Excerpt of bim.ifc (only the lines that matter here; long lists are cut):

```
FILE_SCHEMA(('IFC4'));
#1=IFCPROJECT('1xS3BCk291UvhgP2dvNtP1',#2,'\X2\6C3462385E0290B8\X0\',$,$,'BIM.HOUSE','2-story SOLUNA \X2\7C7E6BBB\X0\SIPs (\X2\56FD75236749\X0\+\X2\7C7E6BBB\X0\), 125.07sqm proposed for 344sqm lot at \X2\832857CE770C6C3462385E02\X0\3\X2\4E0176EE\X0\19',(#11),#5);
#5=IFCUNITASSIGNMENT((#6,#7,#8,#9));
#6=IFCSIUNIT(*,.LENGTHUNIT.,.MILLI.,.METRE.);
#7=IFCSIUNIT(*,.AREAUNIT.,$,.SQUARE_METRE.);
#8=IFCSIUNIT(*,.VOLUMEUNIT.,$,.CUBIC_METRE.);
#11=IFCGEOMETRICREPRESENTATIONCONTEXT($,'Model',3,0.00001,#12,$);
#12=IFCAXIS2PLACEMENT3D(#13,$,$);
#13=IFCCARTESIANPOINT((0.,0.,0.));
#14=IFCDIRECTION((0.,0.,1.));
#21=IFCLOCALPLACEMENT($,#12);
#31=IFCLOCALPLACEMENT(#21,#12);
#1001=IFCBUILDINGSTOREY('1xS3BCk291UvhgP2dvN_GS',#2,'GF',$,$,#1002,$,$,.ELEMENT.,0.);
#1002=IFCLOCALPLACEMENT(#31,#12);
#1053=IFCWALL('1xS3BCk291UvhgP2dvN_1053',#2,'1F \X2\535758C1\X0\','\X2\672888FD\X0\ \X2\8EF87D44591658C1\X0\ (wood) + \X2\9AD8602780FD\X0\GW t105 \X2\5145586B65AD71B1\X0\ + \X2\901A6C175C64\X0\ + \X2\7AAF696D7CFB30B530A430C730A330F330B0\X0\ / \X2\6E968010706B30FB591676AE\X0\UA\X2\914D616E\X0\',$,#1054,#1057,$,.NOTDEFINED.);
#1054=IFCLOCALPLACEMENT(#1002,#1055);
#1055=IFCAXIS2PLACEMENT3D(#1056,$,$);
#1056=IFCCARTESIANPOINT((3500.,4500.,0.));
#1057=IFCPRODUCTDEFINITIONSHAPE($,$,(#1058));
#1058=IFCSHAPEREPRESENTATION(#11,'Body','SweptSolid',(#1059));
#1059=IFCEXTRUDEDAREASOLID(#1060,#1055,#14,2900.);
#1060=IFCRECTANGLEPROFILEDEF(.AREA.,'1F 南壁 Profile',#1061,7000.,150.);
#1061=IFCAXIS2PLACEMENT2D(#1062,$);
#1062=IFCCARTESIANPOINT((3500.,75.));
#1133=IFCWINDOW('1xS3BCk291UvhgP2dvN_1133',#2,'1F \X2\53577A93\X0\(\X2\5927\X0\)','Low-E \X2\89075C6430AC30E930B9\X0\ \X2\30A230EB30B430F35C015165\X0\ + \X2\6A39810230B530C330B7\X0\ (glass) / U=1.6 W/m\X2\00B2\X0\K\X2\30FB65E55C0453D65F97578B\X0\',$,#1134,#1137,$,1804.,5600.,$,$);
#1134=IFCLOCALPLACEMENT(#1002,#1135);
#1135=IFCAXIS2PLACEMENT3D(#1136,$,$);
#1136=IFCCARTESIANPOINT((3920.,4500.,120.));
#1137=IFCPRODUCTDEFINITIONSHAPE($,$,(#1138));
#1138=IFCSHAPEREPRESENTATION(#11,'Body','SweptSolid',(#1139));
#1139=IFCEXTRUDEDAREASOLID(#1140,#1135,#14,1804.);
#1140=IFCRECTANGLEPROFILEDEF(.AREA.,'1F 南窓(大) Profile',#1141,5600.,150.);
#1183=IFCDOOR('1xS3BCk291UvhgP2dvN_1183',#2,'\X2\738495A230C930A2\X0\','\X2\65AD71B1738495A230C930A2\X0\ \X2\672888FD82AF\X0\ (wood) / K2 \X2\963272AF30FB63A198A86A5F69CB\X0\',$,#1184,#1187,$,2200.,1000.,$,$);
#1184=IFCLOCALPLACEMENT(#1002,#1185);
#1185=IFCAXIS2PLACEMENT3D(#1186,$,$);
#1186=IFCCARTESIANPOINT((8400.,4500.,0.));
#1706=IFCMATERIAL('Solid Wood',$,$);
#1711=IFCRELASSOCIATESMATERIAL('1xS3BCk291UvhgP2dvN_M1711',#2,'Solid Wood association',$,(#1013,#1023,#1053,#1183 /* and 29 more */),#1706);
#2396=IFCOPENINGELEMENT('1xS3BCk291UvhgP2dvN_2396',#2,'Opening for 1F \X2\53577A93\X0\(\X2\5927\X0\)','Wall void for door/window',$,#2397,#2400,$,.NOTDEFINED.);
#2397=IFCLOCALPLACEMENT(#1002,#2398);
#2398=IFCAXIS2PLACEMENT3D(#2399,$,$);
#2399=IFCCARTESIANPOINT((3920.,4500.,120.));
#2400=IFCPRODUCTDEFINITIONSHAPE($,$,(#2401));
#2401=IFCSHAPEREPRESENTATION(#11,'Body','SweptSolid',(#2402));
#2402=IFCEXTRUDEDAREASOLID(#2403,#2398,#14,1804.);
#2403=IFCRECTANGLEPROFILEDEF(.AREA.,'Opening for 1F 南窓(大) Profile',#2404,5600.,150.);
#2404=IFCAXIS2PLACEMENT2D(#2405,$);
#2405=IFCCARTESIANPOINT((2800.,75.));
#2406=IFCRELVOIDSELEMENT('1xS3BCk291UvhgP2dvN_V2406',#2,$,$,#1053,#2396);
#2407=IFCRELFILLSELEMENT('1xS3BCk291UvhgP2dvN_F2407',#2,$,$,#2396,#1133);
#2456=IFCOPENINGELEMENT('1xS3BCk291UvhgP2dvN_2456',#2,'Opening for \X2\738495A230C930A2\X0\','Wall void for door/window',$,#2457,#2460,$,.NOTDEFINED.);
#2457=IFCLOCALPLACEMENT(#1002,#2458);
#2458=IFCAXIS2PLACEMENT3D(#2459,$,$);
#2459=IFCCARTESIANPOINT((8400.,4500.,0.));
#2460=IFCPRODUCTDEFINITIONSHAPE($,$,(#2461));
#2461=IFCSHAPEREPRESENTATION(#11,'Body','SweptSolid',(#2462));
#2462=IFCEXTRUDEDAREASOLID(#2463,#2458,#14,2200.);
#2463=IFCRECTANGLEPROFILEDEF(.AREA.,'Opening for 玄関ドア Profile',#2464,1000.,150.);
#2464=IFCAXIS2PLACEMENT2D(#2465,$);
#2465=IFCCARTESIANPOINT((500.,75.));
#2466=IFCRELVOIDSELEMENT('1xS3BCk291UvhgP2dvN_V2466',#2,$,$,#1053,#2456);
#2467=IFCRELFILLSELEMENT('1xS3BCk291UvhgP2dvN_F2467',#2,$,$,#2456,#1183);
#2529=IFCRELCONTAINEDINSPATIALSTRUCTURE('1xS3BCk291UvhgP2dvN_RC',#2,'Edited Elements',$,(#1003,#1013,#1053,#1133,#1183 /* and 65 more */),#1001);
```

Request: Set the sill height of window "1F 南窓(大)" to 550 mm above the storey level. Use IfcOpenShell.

```python
import numpy as np
import ifcopenshell
import ifcopenshell.api.geometry
import ifcopenshell.geom
import ifcopenshell.util.element
import ifcopenshell.util.placement
import ifcopenshell.util.shape
import ifcopenshell.util.unit

model = ifcopenshell.open("bim.ifc")
unit_scale = ifcopenshell.util.unit.calculate_unit_scale(model)

window = model.by_guid("1xS3BCk291UvhgP2dvN_1133")
opening = window.FillsVoids[0].RelatingOpeningElement
storey = ifcopenshell.util.element.get_container(window, ifc_class="IfcBuildingStorey")
level = ifcopenshell.util.placement.get_local_placement(storey.ObjectPlacement)[2, 3]

# The opening's origin need not be at the sill, so measure its lowest point.
shape = ifcopenshell.geom.create_shape(ifcopenshell.geom.settings(), opening)
bottom = ifcopenshell.util.shape.get_shape_bottom_elevation(shape, shape.geometry) / unit_scale
dz = level + 0.55 / unit_scale - bottom

shift = np.array([0.0, 0.0, dz])
# The window is not placed relative to its opening, so move both.
for product in (opening, window):
    matrix = ifcopenshell.util.placement.get_local_placement(product.ObjectPlacement)
    matrix[:3, 3] += shift
    ifcopenshell.api.geometry.edit_object_placement(model, product=product, matrix=matrix, is_si=False)

print(f"moved by {dz * unit_scale:+.3f} m")

model.write("bim_v2.ifc")
```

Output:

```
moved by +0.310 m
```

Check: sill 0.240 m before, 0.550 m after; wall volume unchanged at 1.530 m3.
